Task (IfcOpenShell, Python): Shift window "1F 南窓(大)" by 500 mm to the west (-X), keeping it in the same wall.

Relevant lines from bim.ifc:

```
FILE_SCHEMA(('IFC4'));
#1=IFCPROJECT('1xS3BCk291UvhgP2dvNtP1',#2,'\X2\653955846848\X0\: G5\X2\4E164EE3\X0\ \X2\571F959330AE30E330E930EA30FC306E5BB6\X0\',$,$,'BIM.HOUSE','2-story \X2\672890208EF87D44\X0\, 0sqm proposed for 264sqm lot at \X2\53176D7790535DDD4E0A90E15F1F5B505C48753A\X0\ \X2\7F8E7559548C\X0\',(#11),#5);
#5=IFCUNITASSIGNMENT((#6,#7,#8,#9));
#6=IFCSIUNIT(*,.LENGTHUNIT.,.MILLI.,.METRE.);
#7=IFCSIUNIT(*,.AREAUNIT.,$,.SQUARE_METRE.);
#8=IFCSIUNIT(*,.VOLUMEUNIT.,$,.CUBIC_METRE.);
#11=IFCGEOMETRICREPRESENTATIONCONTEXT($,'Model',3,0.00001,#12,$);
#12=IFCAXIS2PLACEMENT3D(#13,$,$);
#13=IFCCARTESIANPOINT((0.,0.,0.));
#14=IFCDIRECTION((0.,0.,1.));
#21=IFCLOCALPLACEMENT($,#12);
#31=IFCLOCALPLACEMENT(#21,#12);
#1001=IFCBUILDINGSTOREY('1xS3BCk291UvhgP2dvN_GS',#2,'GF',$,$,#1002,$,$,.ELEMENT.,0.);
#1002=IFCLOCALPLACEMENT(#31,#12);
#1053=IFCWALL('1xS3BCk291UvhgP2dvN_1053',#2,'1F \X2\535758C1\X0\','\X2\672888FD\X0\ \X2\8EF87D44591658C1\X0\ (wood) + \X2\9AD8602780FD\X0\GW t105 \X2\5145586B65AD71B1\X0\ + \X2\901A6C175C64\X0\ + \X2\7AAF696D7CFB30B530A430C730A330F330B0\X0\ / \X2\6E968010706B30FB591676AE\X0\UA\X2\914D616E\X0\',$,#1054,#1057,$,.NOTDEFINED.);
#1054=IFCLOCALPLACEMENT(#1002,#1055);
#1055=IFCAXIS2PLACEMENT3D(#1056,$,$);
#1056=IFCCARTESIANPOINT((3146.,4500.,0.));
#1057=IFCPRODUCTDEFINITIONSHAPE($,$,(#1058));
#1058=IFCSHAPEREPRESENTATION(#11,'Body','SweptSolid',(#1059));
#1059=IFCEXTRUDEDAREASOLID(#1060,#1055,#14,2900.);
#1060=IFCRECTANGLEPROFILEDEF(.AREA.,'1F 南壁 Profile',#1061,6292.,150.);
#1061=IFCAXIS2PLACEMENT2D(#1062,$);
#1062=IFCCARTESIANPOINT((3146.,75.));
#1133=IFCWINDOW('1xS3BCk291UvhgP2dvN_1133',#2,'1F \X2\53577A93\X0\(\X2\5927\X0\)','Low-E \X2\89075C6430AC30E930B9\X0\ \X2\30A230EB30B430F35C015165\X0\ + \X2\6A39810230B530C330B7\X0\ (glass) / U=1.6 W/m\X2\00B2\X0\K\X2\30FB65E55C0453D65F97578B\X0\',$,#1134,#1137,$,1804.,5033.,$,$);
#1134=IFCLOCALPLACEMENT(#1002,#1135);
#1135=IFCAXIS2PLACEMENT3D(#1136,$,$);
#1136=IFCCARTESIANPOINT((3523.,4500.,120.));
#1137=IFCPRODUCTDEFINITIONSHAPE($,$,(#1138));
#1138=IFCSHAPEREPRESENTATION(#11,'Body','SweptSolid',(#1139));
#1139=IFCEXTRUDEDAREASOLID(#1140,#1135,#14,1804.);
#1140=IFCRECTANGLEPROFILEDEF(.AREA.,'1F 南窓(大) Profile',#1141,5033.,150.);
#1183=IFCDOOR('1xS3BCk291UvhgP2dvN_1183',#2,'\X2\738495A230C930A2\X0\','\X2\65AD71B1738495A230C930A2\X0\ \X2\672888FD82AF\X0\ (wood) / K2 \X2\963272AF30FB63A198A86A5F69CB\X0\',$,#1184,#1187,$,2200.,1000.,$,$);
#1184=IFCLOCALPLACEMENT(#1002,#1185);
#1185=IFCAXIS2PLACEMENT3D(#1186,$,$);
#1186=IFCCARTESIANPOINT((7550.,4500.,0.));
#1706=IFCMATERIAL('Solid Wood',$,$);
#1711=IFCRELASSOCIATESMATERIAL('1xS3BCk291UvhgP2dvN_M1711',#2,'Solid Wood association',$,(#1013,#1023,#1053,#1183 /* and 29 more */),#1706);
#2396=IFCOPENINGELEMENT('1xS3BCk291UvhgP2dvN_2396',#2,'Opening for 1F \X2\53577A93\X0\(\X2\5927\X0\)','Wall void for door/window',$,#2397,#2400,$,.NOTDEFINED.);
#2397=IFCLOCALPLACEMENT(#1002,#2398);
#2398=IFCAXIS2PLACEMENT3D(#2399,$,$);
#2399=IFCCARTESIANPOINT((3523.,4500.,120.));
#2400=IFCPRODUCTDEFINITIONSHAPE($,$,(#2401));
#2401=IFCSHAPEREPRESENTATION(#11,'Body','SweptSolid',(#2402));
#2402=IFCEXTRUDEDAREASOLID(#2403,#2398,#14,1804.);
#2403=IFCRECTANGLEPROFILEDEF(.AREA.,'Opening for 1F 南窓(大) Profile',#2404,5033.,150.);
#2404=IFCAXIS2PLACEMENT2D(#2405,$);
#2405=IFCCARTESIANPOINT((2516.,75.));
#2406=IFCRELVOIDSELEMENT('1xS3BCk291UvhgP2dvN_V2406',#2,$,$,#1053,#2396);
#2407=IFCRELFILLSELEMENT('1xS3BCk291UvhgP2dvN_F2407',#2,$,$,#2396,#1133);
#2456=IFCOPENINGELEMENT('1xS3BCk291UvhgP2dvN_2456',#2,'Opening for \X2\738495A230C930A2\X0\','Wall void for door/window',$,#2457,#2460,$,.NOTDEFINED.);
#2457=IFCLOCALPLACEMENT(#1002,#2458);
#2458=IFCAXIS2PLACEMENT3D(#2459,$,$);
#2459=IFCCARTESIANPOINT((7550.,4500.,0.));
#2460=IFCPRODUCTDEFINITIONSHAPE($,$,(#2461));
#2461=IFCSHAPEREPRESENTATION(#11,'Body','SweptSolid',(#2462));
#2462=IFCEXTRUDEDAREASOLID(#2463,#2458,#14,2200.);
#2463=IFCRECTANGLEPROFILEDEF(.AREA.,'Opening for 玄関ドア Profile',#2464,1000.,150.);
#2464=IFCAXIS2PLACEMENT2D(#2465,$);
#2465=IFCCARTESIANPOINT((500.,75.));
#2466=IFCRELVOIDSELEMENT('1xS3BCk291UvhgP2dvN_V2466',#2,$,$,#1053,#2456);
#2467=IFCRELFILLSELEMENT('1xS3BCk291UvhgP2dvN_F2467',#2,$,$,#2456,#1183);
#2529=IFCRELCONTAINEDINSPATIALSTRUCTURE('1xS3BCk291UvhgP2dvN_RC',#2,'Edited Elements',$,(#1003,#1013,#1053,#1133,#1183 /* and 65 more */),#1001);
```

```python
import ifcopenshell
import ifcopenshell.api.geometry
import ifcopenshell.util.placement

model = ifcopenshell.open("bim.ifc")

window = model.by_guid("1xS3BCk291UvhgP2dvN_1133")
opening = window.FillsVoids[0].RelatingOpeningElement
wall = opening.VoidsElements[0].RelatingBuildingElement

wall_matrix = ifcopenshell.util.placement.get_local_placement(wall.ObjectPlacement)
shift = wall_matrix[:3, 0] * -500.0
before = ifcopenshell.util.placement.get_local_placement(window.ObjectPlacement)[:3, 3].copy()

# The window is not placed relative to its opening, so move both.
for product in (opening, window):
    matrix = ifcopenshell.util.placement.get_local_placement(product.ObjectPlacement)
    matrix[:3, 3] += shift
    ifcopenshell.api.geometry.edit_object_placement(model, product=product, matrix=matrix, is_si=False)

after = ifcopenshell.util.placement.get_local_placement(window.ObjectPlacement)[:3, 3]
print("window moved by", (after - before).round(3) + 0.0)

model.write("bim_updated.ifc")
```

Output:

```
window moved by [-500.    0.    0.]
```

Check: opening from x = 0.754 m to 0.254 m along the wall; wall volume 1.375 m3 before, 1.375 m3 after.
